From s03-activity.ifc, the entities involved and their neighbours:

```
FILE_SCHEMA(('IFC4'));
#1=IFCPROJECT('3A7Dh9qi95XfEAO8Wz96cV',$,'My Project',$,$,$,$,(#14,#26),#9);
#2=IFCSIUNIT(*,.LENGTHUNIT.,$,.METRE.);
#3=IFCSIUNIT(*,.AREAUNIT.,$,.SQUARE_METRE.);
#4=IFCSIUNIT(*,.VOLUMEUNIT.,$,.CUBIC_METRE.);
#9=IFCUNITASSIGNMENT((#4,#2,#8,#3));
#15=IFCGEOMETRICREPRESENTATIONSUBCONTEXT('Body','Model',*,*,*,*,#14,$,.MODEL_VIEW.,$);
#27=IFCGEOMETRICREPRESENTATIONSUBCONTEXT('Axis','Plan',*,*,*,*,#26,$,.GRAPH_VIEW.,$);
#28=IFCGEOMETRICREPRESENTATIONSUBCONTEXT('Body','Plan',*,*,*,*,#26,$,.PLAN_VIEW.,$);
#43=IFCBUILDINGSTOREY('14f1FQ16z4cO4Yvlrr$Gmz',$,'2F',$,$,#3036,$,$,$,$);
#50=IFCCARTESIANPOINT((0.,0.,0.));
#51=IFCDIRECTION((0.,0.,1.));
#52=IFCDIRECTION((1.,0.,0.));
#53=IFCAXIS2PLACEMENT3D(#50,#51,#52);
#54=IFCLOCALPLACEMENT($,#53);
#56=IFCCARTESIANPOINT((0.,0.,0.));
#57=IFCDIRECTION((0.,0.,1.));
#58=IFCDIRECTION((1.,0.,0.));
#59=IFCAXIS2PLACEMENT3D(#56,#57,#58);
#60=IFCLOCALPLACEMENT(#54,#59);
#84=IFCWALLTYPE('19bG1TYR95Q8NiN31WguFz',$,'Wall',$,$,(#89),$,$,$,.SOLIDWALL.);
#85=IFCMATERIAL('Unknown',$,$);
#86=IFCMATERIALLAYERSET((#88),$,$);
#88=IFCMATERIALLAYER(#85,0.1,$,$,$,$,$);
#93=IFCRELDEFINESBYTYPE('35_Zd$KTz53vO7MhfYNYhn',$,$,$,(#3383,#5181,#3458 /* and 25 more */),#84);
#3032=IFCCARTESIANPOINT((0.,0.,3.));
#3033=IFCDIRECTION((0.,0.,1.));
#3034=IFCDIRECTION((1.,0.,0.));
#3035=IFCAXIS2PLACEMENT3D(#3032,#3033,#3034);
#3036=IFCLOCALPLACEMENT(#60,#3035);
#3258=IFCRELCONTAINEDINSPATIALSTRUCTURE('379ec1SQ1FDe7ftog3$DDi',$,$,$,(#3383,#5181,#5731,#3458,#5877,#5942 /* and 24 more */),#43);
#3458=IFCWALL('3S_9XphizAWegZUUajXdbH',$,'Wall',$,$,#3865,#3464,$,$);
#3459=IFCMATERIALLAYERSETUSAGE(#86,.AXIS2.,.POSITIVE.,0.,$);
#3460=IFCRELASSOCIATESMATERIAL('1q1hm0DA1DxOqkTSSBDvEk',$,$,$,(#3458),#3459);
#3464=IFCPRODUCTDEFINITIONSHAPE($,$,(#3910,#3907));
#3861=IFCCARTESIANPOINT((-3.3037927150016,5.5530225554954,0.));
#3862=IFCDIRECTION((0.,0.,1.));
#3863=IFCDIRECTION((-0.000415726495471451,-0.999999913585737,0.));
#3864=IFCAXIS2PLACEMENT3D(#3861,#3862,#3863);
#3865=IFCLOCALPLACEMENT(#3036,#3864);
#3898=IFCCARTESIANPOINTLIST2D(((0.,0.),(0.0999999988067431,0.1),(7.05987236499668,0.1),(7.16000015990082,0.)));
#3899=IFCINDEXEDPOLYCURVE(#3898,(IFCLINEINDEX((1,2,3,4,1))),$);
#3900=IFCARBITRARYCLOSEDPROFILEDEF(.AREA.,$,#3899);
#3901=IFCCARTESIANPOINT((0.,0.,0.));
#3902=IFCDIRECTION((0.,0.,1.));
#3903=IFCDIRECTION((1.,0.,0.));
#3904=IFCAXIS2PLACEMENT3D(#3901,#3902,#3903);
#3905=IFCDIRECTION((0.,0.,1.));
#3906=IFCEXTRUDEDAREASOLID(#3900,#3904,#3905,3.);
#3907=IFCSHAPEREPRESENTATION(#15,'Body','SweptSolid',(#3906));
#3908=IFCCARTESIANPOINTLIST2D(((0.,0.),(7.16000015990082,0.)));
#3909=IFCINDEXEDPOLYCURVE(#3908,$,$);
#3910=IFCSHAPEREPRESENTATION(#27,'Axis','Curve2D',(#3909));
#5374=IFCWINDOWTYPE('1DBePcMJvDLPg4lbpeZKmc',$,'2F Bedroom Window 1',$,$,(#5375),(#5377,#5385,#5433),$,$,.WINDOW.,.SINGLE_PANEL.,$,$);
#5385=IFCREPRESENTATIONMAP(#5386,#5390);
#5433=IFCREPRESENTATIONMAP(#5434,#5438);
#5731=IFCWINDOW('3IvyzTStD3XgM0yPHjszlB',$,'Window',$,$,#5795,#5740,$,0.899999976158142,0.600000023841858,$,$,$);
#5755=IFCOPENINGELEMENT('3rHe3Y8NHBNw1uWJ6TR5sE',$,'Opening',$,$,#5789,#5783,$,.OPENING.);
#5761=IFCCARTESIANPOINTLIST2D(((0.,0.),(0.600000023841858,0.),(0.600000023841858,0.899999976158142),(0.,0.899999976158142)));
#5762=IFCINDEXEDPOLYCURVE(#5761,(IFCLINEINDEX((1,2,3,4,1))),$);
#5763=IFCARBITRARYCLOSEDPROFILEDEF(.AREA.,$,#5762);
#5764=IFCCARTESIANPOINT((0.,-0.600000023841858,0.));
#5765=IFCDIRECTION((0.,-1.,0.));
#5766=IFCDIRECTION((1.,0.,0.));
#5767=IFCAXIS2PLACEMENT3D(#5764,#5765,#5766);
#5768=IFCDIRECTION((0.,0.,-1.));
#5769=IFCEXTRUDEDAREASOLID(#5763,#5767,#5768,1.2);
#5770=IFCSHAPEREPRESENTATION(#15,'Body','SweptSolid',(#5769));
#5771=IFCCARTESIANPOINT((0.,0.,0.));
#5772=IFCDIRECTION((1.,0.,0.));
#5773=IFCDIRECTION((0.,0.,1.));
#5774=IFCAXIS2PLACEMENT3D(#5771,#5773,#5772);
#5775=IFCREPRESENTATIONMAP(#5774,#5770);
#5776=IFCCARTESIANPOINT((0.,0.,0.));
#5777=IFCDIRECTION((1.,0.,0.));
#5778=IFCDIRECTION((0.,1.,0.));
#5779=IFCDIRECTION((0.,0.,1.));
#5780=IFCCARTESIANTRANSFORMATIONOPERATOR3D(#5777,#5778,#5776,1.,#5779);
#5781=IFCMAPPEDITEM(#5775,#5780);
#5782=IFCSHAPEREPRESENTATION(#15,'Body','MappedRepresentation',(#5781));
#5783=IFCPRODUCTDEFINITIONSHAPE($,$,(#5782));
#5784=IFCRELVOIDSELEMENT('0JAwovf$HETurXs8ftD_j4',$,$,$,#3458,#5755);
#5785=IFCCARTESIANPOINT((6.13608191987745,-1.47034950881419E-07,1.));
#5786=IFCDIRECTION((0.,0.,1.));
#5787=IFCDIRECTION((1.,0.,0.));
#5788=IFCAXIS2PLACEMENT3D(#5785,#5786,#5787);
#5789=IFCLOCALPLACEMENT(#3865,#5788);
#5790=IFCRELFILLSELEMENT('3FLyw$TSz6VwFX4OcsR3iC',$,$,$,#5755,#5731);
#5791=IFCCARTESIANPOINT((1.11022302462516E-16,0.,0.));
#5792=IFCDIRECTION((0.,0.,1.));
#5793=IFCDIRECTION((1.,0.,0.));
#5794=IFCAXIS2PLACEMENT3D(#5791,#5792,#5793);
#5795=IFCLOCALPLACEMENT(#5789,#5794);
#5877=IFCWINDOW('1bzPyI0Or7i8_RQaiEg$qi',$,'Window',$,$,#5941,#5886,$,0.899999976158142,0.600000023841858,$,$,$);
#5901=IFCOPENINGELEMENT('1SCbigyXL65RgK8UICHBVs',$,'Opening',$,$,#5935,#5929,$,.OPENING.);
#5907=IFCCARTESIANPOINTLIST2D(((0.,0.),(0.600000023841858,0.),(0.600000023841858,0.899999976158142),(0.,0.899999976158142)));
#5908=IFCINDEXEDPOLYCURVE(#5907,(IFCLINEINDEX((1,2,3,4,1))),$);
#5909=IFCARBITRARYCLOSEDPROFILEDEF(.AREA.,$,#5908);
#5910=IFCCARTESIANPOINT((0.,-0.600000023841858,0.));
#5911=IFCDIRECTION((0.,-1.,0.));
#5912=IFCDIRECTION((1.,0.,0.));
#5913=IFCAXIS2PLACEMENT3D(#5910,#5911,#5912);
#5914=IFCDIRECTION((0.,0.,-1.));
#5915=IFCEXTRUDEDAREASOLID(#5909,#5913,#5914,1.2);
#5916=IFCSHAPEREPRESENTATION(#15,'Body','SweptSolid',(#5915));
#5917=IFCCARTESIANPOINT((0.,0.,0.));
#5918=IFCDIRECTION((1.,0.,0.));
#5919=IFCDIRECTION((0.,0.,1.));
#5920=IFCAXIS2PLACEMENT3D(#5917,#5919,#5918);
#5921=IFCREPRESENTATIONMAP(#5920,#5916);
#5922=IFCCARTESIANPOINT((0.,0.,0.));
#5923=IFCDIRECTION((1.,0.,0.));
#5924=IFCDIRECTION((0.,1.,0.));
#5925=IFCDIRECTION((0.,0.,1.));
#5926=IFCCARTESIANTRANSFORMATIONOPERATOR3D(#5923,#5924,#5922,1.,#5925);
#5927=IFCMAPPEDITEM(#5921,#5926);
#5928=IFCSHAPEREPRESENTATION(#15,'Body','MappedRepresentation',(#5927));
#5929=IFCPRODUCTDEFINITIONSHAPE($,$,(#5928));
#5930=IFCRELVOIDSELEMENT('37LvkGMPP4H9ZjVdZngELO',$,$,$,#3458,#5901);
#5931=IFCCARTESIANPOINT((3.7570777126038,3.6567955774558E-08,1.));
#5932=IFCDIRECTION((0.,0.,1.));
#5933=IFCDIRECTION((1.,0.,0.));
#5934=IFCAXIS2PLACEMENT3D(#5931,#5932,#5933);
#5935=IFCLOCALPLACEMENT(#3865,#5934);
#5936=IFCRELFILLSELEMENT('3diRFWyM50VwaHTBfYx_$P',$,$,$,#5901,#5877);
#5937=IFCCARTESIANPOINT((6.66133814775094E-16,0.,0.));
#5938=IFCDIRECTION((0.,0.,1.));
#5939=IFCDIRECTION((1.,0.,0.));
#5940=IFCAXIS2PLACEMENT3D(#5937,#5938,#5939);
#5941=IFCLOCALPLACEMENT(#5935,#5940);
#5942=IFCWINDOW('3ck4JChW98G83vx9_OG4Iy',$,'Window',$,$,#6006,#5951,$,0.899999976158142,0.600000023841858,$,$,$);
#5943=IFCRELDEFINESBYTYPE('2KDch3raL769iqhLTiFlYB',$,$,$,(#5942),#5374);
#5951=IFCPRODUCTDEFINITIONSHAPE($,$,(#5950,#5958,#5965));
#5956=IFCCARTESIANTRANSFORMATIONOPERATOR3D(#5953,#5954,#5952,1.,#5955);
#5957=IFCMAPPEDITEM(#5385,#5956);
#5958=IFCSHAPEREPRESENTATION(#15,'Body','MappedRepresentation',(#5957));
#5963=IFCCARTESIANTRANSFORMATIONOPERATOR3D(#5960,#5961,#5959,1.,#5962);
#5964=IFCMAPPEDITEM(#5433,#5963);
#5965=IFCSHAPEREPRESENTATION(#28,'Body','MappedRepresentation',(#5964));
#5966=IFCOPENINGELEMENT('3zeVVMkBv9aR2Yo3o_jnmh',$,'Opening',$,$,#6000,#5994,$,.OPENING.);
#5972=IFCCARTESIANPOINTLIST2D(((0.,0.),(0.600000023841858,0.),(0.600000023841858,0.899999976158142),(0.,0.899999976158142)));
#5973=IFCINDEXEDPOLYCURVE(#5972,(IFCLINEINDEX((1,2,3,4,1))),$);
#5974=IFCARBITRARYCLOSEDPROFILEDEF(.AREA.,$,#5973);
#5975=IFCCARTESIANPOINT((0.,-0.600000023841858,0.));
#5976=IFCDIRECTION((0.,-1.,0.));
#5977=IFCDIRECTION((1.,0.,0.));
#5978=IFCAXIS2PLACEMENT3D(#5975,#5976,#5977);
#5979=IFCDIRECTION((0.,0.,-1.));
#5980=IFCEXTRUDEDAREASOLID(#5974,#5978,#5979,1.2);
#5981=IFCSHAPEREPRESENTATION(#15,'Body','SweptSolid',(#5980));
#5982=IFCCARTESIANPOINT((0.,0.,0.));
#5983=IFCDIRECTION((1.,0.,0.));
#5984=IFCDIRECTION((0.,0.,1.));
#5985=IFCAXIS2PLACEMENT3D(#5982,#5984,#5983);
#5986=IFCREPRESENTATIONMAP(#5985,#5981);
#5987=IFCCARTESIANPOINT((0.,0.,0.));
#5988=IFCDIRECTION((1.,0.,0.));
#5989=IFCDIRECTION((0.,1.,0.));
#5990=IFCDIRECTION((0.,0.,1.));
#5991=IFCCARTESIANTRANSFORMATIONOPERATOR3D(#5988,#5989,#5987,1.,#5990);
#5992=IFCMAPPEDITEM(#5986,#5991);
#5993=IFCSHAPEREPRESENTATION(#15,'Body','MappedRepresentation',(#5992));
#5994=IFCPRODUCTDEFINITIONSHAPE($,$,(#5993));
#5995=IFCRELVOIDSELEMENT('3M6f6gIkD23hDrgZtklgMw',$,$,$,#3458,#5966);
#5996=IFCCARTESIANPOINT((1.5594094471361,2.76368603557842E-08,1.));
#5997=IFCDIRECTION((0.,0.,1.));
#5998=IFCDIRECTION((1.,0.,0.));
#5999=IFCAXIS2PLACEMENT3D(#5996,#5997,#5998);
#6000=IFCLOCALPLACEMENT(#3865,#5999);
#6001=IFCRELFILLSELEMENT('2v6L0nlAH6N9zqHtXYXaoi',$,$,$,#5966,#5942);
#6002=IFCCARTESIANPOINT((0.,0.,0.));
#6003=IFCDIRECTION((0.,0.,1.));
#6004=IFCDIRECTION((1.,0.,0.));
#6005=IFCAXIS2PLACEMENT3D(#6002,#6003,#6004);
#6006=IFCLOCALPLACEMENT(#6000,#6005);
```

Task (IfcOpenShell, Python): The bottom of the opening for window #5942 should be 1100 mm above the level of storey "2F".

```python
import numpy as np
import ifcopenshell
import ifcopenshell.api.geometry
import ifcopenshell.geom
import ifcopenshell.util.element
import ifcopenshell.util.placement
import ifcopenshell.util.shape
import ifcopenshell.util.unit

model = ifcopenshell.open("s03-activity.ifc")
unit_scale = ifcopenshell.util.unit.calculate_unit_scale(model)

window = model.by_guid("3ck4JChW98G83vx9_OG4Iy")
opening = window.FillsVoids[0].RelatingOpeningElement
storey = ifcopenshell.util.element.get_container(window, ifc_class="IfcBuildingStorey")
level = ifcopenshell.util.placement.get_local_placement(storey.ObjectPlacement)[2, 3]

# The opening's origin need not be at the sill, so measure its lowest point.
shape = ifcopenshell.geom.create_shape(ifcopenshell.geom.settings(), opening)
bottom = ifcopenshell.util.shape.get_shape_bottom_elevation(shape, shape.geometry) / unit_scale
dz = level + 1.1 - bottom

shift = np.array([0.0, 0.0, dz])
# The window is placed relative to its opening, so it follows when the opening moves.
matrix = ifcopenshell.util.placement.get_local_placement(opening.ObjectPlacement)
matrix[:3, 3] += shift
ifcopenshell.api.geometry.edit_object_placement(
    model, product=opening, matrix=matrix, is_si=False, should_transform_children=True
)

print(f"moved by {dz * unit_scale:+.3f} m")

model.write("s03-activity_edited.ifc")
```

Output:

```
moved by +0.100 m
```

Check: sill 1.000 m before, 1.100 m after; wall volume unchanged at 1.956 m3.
